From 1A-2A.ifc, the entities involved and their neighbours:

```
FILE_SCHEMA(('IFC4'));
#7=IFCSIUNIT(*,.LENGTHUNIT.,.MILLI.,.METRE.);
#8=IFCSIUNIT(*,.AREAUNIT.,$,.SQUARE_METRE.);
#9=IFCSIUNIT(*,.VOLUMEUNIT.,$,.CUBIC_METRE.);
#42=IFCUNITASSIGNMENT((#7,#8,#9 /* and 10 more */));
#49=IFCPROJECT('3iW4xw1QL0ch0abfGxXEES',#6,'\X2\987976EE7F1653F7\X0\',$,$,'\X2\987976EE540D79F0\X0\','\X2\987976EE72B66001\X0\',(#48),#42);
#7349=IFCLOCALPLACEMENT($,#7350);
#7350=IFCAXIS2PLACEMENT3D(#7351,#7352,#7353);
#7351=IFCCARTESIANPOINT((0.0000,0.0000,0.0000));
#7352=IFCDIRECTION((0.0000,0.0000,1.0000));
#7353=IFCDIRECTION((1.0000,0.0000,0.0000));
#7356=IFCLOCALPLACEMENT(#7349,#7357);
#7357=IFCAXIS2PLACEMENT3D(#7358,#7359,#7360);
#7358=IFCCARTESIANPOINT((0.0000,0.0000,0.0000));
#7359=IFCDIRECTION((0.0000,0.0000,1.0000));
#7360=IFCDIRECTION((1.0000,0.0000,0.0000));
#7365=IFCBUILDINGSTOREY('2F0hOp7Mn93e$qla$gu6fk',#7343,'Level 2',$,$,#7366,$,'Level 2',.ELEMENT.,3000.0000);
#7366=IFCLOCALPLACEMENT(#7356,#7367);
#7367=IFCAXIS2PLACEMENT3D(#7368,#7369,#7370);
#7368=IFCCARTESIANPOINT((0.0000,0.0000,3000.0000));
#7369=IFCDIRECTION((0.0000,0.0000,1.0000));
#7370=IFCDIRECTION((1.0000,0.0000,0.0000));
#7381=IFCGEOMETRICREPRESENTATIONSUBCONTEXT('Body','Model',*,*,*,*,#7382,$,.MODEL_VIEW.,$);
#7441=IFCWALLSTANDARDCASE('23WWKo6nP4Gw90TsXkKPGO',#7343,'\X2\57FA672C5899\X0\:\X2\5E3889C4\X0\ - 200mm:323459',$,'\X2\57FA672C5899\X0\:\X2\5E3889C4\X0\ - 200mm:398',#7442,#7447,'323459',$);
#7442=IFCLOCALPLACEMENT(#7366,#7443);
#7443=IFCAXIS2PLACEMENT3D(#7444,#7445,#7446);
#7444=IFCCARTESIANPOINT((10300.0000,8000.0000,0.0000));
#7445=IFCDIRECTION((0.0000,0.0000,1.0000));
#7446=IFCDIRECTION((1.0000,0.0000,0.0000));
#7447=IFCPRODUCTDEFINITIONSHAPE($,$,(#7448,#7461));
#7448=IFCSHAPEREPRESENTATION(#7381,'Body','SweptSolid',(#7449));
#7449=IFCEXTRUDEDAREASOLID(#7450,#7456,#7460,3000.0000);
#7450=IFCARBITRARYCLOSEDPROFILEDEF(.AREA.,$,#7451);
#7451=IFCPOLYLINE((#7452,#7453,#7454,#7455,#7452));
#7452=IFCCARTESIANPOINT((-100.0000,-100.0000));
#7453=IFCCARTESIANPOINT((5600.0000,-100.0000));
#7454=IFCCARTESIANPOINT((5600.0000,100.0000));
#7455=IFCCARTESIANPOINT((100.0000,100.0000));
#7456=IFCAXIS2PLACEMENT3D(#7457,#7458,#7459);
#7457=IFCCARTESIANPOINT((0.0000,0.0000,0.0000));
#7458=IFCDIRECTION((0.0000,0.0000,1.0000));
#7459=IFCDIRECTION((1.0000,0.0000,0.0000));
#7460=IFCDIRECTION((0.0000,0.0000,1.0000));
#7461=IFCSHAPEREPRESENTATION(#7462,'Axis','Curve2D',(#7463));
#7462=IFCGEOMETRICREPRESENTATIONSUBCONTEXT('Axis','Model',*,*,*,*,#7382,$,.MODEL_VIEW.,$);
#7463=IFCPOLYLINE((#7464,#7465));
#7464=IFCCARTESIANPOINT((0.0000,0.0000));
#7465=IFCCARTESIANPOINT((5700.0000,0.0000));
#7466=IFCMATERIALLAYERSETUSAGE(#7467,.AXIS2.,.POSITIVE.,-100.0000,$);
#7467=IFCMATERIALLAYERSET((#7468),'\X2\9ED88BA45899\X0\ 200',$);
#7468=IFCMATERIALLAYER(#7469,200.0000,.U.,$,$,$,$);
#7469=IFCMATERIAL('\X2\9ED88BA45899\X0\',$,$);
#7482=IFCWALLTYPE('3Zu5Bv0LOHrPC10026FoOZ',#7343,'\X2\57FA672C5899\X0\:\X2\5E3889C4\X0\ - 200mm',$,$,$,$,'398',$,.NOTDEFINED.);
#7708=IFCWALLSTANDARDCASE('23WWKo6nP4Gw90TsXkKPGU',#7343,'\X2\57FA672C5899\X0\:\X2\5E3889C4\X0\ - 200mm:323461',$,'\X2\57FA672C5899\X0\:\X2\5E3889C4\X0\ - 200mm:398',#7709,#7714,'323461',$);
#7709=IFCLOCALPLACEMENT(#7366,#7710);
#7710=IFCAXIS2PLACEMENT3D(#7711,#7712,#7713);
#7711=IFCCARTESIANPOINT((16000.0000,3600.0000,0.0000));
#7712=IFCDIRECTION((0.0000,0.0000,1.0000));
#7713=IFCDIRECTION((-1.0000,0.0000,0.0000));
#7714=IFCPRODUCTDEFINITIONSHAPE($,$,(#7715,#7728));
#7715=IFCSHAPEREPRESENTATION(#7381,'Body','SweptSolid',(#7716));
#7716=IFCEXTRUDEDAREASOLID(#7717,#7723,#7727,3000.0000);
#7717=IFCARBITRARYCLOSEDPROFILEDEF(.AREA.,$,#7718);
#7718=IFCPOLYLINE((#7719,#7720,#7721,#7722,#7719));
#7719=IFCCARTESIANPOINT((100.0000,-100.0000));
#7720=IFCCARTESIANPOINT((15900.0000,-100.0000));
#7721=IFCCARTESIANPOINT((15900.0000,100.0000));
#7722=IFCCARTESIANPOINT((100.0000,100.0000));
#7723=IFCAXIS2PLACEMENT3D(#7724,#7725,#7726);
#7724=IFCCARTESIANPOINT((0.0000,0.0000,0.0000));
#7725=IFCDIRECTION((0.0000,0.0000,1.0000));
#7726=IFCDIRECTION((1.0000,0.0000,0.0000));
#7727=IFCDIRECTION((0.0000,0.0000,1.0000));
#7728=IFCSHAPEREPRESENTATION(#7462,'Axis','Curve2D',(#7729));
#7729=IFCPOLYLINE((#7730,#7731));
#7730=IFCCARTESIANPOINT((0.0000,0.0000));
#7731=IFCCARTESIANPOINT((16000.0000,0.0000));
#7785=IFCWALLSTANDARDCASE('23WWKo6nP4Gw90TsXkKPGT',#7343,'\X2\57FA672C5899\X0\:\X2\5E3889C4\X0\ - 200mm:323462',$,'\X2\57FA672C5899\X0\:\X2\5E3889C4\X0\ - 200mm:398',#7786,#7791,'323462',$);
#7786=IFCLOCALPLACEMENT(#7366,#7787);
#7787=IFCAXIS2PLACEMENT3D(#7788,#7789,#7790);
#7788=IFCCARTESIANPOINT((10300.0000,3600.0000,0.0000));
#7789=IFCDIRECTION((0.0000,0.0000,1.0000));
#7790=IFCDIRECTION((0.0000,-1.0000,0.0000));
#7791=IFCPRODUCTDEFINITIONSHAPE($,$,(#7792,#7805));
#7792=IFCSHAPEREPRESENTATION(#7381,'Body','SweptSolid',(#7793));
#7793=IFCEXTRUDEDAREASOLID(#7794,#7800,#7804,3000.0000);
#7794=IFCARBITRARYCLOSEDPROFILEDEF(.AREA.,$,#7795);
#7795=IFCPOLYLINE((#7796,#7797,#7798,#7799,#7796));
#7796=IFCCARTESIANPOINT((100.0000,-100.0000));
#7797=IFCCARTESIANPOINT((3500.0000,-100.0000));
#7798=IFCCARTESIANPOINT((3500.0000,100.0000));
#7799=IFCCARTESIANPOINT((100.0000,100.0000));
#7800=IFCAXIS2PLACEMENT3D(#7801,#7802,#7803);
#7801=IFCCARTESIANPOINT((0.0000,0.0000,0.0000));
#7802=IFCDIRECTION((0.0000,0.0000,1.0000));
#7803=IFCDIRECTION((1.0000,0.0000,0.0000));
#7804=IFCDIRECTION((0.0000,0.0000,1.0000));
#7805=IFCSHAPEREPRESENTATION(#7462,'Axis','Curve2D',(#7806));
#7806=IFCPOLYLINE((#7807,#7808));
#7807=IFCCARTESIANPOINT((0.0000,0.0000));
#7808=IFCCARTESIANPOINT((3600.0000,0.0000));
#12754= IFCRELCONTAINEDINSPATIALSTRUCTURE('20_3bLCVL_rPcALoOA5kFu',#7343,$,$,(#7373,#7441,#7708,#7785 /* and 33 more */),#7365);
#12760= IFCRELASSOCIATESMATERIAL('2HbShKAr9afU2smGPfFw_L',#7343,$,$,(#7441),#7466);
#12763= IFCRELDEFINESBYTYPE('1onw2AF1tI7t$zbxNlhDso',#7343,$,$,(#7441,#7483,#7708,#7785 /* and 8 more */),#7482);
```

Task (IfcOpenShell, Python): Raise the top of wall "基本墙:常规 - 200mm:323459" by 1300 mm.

```python
import ifcopenshell
import ifcopenshell.geom
import ifcopenshell.util.representation
import ifcopenshell.util.shape
import ifcopenshell.util.unit

model = ifcopenshell.open("1A-2A.ifc")
unit_scale = ifcopenshell.util.unit.calculate_unit_scale(model)
settings = ifcopenshell.geom.settings()


def volume(element):
    """Net volume in cubic metres, openings subtracted."""
    shape = ifcopenshell.geom.create_shape(settings, element)
    return ifcopenshell.util.shape.get_volume(shape.geometry)


wall = model.by_id(7441)
before = volume(wall)

body = ifcopenshell.util.representation.get_representation(wall, "Model", "Body")
solid = body.Items[0]
old_height = solid.Depth
solid.Depth += 1.3 / unit_scale
after = volume(wall)

print(f"height {old_height:g} -> {solid.Depth:g}, volume {before:.3f} -> {after:.3f} m3")

model.write("1A-2A_v2.ifc")
```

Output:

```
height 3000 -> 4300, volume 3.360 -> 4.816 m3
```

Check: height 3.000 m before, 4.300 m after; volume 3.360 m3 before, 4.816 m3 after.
